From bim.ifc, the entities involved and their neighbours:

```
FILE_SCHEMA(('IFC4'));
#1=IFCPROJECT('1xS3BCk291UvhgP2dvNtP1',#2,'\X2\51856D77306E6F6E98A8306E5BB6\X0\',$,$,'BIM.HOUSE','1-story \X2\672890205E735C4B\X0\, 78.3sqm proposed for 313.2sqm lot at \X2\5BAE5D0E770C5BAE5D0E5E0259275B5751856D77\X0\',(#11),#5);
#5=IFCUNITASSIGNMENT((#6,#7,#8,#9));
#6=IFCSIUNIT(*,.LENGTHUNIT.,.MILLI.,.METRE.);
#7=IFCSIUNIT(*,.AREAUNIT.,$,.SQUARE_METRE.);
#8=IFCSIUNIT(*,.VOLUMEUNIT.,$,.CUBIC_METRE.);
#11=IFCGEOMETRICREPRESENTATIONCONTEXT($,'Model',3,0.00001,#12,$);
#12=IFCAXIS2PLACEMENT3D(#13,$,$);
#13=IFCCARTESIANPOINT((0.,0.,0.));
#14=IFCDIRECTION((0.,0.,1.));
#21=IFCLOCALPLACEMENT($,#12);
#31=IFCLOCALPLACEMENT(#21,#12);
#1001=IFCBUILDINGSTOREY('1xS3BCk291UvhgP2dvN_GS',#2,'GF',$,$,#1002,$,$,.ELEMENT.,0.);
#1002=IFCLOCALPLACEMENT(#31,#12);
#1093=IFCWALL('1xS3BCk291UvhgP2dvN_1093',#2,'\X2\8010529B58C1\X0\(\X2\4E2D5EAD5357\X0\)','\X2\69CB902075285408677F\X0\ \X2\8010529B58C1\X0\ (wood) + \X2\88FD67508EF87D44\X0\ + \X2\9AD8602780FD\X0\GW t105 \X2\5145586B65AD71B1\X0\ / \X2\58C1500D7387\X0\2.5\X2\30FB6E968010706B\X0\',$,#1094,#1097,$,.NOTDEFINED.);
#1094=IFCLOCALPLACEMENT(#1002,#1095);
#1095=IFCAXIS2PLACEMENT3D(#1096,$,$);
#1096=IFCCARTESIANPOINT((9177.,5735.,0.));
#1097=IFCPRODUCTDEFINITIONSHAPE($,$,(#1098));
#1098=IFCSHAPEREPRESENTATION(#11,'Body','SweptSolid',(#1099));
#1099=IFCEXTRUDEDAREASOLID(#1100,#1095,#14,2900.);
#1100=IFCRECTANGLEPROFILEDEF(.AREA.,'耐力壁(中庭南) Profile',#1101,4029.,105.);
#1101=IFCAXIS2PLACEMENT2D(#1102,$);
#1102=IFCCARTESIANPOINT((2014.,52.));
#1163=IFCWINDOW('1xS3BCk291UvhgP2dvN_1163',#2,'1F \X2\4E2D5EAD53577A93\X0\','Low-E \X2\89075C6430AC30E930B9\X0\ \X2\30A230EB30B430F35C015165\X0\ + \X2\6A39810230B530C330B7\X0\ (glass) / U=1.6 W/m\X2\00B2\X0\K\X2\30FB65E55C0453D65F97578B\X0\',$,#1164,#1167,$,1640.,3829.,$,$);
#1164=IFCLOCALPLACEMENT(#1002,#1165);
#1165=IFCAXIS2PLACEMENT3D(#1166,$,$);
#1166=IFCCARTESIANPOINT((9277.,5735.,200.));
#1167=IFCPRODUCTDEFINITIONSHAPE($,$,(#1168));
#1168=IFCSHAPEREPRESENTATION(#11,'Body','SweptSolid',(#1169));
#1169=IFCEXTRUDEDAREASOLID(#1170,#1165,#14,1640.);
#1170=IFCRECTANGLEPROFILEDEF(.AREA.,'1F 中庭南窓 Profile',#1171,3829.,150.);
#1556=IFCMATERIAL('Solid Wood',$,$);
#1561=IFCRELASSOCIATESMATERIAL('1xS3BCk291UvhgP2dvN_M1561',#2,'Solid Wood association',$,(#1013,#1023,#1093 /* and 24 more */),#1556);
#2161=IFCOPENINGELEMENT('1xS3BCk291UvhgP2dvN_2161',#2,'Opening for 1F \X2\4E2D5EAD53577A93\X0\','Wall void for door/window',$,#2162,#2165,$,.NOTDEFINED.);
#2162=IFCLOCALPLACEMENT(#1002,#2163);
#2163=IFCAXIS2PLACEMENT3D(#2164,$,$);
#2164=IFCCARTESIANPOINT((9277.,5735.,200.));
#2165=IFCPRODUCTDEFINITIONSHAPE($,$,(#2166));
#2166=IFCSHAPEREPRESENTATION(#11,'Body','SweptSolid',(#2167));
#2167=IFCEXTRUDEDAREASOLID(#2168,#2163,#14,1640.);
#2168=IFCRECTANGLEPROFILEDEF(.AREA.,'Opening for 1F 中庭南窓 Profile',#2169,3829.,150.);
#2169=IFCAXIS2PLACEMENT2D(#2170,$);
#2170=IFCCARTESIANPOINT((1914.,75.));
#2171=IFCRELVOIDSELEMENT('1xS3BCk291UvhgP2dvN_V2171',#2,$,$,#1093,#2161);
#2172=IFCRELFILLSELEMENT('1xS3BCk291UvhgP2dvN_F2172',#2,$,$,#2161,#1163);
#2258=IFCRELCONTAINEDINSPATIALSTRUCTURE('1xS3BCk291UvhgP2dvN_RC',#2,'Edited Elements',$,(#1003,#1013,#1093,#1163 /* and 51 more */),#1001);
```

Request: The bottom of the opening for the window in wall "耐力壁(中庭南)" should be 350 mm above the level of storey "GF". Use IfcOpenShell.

```python
import numpy as np
import ifcopenshell
import ifcopenshell.api.geometry
import ifcopenshell.geom
import ifcopenshell.util.element
import ifcopenshell.util.placement
import ifcopenshell.util.shape
import ifcopenshell.util.unit

model = ifcopenshell.open("bim.ifc")
unit_scale = ifcopenshell.util.unit.calculate_unit_scale(model)

window = model.by_guid("1xS3BCk291UvhgP2dvN_1163")
opening = window.FillsVoids[0].RelatingOpeningElement
storey = ifcopenshell.util.element.get_container(window, ifc_class="IfcBuildingStorey")
level = ifcopenshell.util.placement.get_local_placement(storey.ObjectPlacement)[2, 3]

# The opening's origin need not be at the sill, so measure its lowest point.
shape = ifcopenshell.geom.create_shape(ifcopenshell.geom.settings(), opening)
bottom = ifcopenshell.util.shape.get_shape_bottom_elevation(shape, shape.geometry) / unit_scale
dz = level + 350.0 - bottom

shift = np.array([0.0, 0.0, dz])
# The window is not placed relative to its opening, so move both.
for product in (opening, window):
    matrix = ifcopenshell.util.placement.get_local_placement(product.ObjectPlacement)
    matrix[:3, 3] += shift
    ifcopenshell.api.geometry.edit_object_placement(model, product=product, matrix=matrix, is_si=False)

print(f"moved by {dz * unit_scale:+.3f} m")

model.write("bim_rev.ifc")
```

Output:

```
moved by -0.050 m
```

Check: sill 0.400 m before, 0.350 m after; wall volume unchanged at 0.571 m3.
